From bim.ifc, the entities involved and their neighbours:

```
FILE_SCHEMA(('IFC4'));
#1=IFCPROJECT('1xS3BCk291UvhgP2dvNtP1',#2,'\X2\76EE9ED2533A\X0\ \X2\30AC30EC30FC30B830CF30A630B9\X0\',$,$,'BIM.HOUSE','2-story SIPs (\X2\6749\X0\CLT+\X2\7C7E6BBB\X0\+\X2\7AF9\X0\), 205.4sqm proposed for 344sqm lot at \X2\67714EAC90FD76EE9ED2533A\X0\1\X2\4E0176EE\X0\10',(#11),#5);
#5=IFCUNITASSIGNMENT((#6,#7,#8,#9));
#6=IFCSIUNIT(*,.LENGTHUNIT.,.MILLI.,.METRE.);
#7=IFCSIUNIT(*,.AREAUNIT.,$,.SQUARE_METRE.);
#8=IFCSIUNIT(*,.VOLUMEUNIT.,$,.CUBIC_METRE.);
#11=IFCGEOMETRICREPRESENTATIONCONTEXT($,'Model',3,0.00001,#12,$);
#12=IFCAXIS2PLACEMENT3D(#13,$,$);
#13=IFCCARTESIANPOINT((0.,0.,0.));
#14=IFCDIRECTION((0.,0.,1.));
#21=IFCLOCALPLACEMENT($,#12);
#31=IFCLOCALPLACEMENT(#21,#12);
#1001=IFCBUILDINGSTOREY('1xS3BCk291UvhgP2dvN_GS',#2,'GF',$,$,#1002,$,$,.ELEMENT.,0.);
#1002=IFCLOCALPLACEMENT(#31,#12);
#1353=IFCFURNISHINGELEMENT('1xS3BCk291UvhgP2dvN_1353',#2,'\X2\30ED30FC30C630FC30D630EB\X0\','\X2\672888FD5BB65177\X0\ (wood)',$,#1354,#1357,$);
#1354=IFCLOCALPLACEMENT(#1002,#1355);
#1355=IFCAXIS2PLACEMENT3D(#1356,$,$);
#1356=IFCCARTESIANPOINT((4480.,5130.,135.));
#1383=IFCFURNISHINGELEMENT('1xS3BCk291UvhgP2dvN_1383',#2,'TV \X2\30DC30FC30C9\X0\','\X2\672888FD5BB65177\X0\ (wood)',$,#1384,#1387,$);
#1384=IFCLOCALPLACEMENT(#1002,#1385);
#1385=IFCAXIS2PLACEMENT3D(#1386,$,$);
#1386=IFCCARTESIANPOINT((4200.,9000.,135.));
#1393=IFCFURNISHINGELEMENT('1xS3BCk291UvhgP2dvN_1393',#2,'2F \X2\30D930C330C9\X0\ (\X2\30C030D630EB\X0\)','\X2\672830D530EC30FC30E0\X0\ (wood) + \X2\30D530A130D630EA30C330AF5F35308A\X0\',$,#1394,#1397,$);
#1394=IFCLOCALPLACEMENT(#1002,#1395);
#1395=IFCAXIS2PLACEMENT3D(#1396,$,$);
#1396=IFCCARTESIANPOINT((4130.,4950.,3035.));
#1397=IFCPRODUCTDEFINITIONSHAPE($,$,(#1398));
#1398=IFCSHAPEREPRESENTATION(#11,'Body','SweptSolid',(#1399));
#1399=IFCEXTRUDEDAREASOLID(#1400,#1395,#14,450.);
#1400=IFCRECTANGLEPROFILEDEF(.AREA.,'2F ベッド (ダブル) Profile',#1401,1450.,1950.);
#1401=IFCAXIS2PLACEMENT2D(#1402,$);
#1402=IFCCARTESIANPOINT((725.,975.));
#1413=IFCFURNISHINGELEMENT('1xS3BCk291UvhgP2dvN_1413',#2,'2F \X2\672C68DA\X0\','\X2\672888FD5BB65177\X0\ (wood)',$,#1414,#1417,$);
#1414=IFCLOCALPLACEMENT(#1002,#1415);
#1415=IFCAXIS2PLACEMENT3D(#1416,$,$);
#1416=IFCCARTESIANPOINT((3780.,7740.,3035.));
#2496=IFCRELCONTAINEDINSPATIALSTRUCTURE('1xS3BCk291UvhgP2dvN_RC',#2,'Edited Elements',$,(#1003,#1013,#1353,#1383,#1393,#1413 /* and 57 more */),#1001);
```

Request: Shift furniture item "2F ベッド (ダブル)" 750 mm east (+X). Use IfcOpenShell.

```python
import ifcopenshell
import ifcopenshell.api.geometry
import ifcopenshell.util.placement
import ifcopenshell.util.unit

model = ifcopenshell.open("bim.ifc")
unit_scale = ifcopenshell.util.unit.calculate_unit_scale(model)

item = model.by_guid("1xS3BCk291UvhgP2dvN_1393")
matrix = ifcopenshell.util.placement.get_local_placement(item.ObjectPlacement)
matrix[0, 3] += 0.75 / unit_scale
ifcopenshell.api.geometry.edit_object_placement(model, product=item, matrix=matrix, is_si=False)

print(ifcopenshell.util.placement.get_local_placement(item.ObjectPlacement).round(3) + 0.0)

model.write("bim_updated.ifc")
```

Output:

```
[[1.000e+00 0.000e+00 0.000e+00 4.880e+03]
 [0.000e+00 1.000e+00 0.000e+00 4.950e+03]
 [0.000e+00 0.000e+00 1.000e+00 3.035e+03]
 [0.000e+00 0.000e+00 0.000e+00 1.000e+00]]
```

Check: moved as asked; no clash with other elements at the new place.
